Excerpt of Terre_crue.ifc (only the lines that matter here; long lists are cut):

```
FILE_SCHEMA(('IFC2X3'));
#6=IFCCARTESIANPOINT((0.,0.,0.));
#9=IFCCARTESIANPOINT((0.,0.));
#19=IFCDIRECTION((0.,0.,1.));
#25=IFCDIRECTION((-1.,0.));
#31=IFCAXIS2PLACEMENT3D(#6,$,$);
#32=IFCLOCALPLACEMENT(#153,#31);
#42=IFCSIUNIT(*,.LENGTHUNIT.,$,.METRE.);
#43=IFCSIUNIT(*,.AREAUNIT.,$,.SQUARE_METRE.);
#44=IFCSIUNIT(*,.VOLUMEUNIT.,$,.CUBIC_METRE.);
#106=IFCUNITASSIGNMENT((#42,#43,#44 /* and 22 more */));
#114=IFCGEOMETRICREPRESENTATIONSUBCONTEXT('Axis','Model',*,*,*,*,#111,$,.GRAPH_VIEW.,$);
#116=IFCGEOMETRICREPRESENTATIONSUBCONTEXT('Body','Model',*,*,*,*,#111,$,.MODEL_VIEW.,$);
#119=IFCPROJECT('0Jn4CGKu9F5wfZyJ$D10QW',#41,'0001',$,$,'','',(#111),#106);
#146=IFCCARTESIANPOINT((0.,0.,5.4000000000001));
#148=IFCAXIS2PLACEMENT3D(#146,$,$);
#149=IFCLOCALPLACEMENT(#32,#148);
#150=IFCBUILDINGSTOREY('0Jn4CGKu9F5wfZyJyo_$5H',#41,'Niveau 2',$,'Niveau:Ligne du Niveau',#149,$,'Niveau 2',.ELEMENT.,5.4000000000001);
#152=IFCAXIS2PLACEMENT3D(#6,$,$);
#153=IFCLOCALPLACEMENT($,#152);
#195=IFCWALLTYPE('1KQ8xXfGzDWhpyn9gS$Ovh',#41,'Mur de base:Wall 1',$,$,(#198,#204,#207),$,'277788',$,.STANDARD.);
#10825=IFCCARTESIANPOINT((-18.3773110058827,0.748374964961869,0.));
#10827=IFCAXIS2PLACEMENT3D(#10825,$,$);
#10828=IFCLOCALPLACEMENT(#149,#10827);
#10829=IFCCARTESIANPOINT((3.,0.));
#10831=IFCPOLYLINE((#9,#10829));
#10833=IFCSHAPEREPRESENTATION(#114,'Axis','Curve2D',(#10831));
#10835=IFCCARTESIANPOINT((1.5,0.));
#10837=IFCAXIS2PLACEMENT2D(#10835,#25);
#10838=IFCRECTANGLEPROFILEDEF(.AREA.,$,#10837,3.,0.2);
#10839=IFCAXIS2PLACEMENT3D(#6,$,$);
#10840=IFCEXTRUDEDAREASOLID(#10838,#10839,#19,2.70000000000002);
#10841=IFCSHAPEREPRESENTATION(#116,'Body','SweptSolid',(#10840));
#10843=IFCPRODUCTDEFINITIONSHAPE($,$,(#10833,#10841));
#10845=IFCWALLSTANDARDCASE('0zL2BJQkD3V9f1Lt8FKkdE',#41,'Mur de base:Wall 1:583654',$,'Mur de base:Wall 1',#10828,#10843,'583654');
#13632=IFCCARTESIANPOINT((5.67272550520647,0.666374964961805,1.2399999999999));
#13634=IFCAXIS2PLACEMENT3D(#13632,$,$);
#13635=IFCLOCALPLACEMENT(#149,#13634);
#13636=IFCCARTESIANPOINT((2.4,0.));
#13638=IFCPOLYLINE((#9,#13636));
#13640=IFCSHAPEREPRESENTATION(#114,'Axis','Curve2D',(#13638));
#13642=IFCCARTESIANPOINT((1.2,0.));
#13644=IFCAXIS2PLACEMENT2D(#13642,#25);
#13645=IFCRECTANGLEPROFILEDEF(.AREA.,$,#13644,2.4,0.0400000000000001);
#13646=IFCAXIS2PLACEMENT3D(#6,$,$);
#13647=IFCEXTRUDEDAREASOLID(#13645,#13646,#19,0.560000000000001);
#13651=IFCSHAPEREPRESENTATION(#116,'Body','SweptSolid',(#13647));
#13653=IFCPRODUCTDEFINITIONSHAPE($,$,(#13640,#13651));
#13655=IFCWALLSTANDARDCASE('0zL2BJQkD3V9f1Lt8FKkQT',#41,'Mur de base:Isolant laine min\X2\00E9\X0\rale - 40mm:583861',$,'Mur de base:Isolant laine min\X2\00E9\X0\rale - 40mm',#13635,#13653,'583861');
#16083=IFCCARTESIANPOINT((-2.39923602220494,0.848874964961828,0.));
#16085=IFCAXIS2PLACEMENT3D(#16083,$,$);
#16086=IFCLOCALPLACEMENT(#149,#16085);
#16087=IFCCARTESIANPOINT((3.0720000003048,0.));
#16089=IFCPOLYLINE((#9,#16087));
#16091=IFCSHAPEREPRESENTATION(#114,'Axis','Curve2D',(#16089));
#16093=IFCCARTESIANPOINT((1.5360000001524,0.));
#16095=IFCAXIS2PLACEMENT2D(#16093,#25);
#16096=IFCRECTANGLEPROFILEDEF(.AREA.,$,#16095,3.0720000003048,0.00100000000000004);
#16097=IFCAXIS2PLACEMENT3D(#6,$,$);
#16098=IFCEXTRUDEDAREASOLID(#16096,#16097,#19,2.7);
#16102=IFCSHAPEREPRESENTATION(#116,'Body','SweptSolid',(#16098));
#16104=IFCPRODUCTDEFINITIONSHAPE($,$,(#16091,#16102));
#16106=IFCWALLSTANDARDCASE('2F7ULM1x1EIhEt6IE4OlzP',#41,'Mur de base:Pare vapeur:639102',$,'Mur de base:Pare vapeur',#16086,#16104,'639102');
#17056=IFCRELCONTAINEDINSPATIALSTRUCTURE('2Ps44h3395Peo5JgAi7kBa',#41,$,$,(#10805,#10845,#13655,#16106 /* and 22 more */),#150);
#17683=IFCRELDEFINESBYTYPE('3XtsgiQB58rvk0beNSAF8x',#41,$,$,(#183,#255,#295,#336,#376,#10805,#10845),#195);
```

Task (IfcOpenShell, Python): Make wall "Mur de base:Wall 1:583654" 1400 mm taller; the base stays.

```python
import ifcopenshell
import ifcopenshell.geom
import ifcopenshell.util.representation
import ifcopenshell.util.shape
import ifcopenshell.util.unit

model = ifcopenshell.open("Terre_crue.ifc")
unit_scale = ifcopenshell.util.unit.calculate_unit_scale(model)
settings = ifcopenshell.geom.settings()


def volume(element):
    """Net volume in cubic metres, openings subtracted."""
    shape = ifcopenshell.geom.create_shape(settings, element)
    return ifcopenshell.util.shape.get_volume(shape.geometry)


wall = model.by_id(10845)
before = volume(wall)

body = ifcopenshell.util.representation.get_representation(wall, "Model", "Body")
solid = body.Items[0]
old_height = solid.Depth
solid.Depth += 1.4 / unit_scale
after = volume(wall)

print(f"height {old_height:g} -> {solid.Depth:g}, volume {before:.3f} -> {after:.3f} m3")

model.write("Terre_crue_edited.ifc")
```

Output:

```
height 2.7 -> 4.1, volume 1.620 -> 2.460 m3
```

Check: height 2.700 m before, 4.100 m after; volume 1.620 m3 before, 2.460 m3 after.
